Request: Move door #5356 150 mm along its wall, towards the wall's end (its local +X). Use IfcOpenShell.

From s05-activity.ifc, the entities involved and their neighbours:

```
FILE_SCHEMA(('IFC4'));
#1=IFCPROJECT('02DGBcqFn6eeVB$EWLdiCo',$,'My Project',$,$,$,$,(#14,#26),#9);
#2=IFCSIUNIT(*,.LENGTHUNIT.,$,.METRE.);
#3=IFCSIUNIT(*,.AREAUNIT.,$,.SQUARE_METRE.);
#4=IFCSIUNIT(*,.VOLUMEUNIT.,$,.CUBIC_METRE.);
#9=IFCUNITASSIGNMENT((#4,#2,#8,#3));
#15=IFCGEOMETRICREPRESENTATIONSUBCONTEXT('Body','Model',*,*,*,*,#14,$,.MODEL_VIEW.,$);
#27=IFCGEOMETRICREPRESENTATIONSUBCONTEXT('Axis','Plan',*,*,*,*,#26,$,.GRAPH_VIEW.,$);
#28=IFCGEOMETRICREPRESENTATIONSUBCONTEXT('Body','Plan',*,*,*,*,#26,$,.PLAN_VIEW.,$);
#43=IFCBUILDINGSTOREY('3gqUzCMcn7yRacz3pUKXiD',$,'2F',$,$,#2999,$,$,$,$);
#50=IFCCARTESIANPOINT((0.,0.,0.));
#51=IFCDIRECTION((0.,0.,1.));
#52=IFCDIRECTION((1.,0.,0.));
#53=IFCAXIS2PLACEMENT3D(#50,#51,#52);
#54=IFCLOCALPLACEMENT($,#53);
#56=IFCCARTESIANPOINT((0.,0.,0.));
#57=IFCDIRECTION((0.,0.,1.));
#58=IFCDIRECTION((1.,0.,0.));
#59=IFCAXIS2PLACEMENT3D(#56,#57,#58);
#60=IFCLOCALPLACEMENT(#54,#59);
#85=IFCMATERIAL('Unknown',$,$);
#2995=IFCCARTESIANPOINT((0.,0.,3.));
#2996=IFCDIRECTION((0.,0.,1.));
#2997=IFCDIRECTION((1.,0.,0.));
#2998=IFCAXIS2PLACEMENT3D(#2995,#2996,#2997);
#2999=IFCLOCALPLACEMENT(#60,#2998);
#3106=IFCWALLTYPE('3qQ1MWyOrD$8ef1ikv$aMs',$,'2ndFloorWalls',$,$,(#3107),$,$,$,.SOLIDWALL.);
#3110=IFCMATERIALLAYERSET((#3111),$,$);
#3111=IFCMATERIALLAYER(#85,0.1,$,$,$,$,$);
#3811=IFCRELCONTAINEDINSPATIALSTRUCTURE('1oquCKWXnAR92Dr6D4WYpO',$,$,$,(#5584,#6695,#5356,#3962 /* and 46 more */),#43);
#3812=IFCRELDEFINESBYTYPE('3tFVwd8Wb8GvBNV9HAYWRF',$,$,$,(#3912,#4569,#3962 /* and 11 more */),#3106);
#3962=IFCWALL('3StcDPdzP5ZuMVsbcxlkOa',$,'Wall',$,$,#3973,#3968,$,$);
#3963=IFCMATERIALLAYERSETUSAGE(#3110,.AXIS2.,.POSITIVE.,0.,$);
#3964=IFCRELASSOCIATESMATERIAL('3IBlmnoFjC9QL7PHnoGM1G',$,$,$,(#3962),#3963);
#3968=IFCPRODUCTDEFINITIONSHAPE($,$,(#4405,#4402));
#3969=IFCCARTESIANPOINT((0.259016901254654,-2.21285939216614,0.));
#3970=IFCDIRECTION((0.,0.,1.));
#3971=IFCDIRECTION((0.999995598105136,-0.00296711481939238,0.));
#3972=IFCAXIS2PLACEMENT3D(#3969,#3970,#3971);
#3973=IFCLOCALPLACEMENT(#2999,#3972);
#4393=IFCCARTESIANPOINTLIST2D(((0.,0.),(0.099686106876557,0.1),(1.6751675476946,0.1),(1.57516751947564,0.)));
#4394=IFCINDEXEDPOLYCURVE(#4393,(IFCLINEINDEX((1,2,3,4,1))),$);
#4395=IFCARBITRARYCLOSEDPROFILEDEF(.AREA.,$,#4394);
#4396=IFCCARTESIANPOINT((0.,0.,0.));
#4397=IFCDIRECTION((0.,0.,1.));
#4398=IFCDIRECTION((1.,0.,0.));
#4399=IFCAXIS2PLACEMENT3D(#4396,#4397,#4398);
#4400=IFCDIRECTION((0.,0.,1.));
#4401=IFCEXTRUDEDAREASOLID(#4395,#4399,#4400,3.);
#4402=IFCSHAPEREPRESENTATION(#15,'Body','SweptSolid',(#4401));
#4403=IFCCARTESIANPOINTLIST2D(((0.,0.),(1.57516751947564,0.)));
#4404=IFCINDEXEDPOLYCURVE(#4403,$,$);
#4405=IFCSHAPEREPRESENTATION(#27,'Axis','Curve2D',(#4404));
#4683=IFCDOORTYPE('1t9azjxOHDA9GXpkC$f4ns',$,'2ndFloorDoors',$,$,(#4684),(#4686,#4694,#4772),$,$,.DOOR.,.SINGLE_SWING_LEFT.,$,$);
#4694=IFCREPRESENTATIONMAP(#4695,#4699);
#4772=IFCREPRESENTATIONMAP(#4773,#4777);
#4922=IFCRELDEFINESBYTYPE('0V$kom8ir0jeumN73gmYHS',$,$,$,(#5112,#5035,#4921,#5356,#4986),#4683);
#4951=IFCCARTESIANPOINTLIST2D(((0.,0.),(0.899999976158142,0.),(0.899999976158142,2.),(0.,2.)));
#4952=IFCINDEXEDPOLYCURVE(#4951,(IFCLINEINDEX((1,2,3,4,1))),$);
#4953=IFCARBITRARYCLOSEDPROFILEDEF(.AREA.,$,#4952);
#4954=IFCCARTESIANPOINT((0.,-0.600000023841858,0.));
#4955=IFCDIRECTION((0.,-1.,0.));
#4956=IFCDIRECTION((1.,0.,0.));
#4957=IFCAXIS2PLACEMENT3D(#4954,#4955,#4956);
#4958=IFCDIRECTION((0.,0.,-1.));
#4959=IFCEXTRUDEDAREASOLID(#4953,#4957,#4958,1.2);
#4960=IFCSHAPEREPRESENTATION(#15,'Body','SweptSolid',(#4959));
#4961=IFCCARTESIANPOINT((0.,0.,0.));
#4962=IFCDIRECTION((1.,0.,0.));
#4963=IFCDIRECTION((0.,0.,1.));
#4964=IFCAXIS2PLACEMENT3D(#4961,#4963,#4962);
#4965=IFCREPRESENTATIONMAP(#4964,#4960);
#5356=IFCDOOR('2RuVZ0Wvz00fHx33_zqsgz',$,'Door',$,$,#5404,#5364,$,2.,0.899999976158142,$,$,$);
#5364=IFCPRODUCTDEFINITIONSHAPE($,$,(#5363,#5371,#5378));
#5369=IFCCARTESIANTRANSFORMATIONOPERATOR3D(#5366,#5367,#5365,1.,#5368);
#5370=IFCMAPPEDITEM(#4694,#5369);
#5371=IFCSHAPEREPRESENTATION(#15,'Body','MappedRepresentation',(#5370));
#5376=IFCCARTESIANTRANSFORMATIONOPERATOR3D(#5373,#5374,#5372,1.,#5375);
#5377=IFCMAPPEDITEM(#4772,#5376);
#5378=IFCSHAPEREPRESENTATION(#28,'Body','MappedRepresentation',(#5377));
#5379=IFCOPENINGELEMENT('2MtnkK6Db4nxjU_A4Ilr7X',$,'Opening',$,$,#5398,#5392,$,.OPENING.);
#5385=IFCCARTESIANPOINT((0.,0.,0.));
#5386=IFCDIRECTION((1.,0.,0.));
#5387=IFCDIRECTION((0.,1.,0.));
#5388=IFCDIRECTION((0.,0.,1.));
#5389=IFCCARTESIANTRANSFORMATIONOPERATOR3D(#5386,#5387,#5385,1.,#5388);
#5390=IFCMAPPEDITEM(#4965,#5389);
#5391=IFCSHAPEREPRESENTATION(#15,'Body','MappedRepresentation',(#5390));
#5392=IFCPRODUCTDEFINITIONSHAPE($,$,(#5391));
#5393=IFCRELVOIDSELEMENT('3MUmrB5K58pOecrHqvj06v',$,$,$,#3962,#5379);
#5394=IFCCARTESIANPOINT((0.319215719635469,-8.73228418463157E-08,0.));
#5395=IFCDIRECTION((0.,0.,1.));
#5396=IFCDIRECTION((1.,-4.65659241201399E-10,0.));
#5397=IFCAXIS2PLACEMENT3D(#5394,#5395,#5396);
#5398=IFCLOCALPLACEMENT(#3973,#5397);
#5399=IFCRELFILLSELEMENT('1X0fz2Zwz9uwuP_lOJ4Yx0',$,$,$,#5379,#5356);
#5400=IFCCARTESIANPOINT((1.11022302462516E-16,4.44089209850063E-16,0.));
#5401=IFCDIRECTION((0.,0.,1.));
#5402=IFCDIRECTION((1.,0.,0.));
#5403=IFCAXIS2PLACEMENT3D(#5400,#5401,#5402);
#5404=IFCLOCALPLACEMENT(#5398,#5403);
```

```python
import ifcopenshell
import ifcopenshell.api.geometry
import ifcopenshell.util.placement
import ifcopenshell.util.unit

model = ifcopenshell.open("s05-activity.ifc")
unit_scale = ifcopenshell.util.unit.calculate_unit_scale(model)

door = model.by_guid("2RuVZ0Wvz00fHx33_zqsgz")
opening = door.FillsVoids[0].RelatingOpeningElement
wall = opening.VoidsElements[0].RelatingBuildingElement

wall_matrix = ifcopenshell.util.placement.get_local_placement(wall.ObjectPlacement)
shift = wall_matrix[:3, 0] * 0.15 / unit_scale
before = ifcopenshell.util.placement.get_local_placement(door.ObjectPlacement)[:3, 3].copy()

# The door is placed relative to its opening, so it follows when the opening moves.
matrix = ifcopenshell.util.placement.get_local_placement(opening.ObjectPlacement)
matrix[:3, 3] += shift
ifcopenshell.api.geometry.edit_object_placement(
    model, product=opening, matrix=matrix, is_si=False, should_transform_children=True
)

after = ifcopenshell.util.placement.get_local_placement(door.ObjectPlacement)[:3, 3]
print("door moved by", (after - before).round(3) + 0.0)

model.write("s05-activity_edited.ifc")
```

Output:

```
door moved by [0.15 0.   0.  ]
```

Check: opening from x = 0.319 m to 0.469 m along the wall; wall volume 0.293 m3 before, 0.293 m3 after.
